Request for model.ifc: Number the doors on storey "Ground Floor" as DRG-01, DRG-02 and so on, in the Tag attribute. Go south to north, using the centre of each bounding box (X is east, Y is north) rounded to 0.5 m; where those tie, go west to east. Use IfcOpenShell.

First a look at what the model holds.

```python
import ifcopenshell
import ifcopenshell.util.element
import ifcopenshell.util.placement

model = ifcopenshell.open("model.ifc")
print(model.schema)
storey = next(s for s in model.by_type("IfcBuildingStorey") if s.Name == "Ground Floor")
doors = [e for e in ifcopenshell.util.element.get_decomposition(storey) if e.is_a("IfcDoor")]
for e in sorted(doors, key=lambda e: e.id()):
    origin = ifcopenshell.util.placement.get_local_placement(e.ObjectPlacement)[:3, 3]
    print(e.id(), e.Tag, e.Name, origin.round(2) + 0.0, sep=" | ")
```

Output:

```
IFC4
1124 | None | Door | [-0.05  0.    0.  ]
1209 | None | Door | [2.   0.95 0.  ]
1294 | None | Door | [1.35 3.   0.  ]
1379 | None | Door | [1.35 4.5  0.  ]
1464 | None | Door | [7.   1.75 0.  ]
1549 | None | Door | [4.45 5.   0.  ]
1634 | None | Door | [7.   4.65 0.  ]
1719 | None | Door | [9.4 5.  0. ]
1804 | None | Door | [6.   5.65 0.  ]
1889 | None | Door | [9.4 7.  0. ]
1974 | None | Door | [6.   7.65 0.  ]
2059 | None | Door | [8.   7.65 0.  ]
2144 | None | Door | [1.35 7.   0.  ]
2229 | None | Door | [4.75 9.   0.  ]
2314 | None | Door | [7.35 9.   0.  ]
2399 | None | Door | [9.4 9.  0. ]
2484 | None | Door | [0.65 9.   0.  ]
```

```python
import ifcopenshell
import ifcopenshell.geom
import ifcopenshell.util.element
import ifcopenshell.util.shape

model = ifcopenshell.open("model.ifc")
settings = ifcopenshell.geom.settings()
settings.set("use-world-coords", True)


def centre(element):
    shape = ifcopenshell.geom.create_shape(settings, element)
    return ifcopenshell.util.shape.get_bbox_centroid(shape.geometry)


storey = next(s for s in model.by_type("IfcBuildingStorey") if s.Name == "Ground Floor")
doors = [e for e in ifcopenshell.util.element.get_decomposition(storey) if e.is_a("IfcDoor")]

# Insertion points can sit at a corner or the storey origin, so sort by the geometry (in metres).
centres = {e: centre(e) for e in doors}
doors.sort(key=lambda e: (round(centres[e][1] / 0.5), centres[e][0]))

for i, e in enumerate(doors, start=1):
    number = f"DRG-{i:02d}"
    e.Tag = number
    print(e.id(), number)

model.write("model_updated.ifc")
```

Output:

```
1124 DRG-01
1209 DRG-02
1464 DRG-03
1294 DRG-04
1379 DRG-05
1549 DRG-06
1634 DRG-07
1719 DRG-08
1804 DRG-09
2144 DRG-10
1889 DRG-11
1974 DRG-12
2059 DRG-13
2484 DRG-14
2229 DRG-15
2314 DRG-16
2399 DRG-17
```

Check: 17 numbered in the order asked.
